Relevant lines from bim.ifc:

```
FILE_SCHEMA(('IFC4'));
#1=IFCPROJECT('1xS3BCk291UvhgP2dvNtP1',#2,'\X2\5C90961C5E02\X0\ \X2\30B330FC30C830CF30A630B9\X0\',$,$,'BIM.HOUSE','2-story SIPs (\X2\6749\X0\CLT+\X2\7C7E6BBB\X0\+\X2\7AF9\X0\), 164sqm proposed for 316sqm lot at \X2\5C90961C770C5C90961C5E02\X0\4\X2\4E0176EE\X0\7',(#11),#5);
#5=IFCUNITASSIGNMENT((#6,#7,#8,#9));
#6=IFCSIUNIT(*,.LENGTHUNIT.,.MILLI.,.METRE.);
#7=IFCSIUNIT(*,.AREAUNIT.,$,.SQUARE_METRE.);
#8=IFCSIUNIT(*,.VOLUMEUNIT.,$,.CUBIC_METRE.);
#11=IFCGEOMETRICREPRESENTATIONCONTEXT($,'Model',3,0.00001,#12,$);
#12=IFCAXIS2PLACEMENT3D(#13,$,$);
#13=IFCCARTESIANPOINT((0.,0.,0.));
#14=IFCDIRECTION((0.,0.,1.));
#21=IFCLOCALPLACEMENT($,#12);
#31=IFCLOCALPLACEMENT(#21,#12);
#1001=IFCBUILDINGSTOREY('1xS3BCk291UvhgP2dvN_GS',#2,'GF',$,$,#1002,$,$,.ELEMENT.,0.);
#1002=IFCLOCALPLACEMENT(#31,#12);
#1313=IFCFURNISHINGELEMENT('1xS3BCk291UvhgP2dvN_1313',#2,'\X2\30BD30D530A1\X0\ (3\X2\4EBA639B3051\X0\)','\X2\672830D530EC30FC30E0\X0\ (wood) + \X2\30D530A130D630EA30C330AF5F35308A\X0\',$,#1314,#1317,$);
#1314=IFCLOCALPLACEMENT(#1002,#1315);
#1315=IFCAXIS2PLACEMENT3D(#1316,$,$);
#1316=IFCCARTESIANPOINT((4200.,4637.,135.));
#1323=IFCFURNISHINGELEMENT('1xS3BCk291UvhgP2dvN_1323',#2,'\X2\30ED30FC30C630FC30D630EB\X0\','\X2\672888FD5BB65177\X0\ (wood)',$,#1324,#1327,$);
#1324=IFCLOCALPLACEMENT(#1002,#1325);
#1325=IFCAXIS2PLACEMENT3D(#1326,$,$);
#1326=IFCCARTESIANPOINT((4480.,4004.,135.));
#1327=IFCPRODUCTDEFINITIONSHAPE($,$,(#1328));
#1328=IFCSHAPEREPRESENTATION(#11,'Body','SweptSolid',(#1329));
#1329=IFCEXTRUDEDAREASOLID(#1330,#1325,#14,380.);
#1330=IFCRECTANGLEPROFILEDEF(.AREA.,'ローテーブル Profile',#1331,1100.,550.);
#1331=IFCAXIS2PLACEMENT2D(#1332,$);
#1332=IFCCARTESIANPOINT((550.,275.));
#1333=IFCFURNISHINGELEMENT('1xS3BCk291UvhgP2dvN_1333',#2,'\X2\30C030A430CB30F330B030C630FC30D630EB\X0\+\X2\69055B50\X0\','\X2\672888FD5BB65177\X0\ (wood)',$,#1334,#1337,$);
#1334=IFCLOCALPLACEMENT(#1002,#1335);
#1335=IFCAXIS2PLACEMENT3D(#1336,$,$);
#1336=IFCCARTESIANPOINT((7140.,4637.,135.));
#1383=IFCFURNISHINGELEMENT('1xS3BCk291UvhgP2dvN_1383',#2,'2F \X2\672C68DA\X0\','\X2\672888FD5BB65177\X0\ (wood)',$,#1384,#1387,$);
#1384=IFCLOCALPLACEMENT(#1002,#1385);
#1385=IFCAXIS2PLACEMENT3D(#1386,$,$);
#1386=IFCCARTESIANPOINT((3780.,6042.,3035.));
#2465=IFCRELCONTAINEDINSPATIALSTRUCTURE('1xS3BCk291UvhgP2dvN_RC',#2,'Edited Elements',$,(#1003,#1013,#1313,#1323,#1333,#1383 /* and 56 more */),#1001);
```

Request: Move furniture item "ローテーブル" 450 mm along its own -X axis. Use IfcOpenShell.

```python
import ifcopenshell
import ifcopenshell.api.geometry
import ifcopenshell.util.placement

model = ifcopenshell.open("bim.ifc")

item = model.by_id(1323)
matrix = ifcopenshell.util.placement.get_local_placement(item.ObjectPlacement)
matrix[:3, 3] -= matrix[:3, 0] * 450.0
ifcopenshell.api.geometry.edit_object_placement(model, product=item, matrix=matrix, is_si=False)

print(ifcopenshell.util.placement.get_local_placement(item.ObjectPlacement).round(3) + 0.0)

model.write("bim_edited.ifc")
```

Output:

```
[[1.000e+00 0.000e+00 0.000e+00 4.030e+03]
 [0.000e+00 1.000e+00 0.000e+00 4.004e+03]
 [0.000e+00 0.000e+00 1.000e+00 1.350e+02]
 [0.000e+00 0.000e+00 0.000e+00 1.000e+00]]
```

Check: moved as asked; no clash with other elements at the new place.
